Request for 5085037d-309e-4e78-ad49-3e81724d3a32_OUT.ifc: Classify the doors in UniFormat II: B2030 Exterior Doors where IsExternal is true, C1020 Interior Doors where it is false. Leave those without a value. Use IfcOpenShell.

First a look at what the model holds.

```python
import ifcopenshell
import ifcopenshell.util.element

model = ifcopenshell.open("5085037d-309e-4e78-ad49-3e81724d3a32_OUT.ifc")
print(model.schema)
print("classifications:", [c.Name for c in model.by_type("IfcClassification")])
values = [ifcopenshell.util.element.get_pset(e, "Pset_DoorCommon", "IsExternal") for e in model.by_type("IfcDoor")]
for value in (True, False, None):
    print("IsExternal", value, values.count(value))
```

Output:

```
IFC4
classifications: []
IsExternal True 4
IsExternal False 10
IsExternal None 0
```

```python
import ifcopenshell
import ifcopenshell.api.classification
import ifcopenshell.util.element

model = ifcopenshell.open("5085037d-309e-4e78-ad49-3e81724d3a32_OUT.ifc")

system = ifcopenshell.api.classification.add_classification(model, classification="UniFormat II")

doors = model.by_type("IfcDoor")
external = {e: ifcopenshell.util.element.get_pset(e, "Pset_DoorCommon", "IsExternal") for e in doors}
for flag, code, name in ((True, "B2030", "Exterior Doors"), (False, "C1020", "Interior Doors")):
    products = [e for e in doors if external[e] is flag]
    ifcopenshell.api.classification.add_reference(
        model, products=products, classification=system, identification=code, name=name
    )
    print(code, len(products))

model.write("5085037d-309e-4e78-ad49-3e81724d3a32_OUT_rev.ifc")
```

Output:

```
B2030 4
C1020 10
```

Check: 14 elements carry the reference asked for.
